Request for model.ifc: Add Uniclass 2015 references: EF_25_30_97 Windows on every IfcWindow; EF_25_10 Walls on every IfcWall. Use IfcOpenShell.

First a look at what the model holds.

```python
import ifcopenshell

model = ifcopenshell.open("model.ifc")
print(model.schema)
print("classifications:", [c.Name for c in model.by_type("IfcClassification")])
for ifc_class in ("IfcDoor", "IfcRoof", "IfcStair", "IfcWall", "IfcWindow"):
    print(ifc_class, len(model.by_type(ifc_class)))
```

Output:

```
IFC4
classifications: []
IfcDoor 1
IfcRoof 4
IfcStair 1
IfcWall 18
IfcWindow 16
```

```python
import ifcopenshell
import ifcopenshell.api.classification

model = ifcopenshell.open("model.ifc")

system = ifcopenshell.api.classification.add_classification(model, classification="Uniclass 2015")

codes = {
    "IfcWindow": ("EF_25_30_97", "Windows"),
    "IfcWall": ("EF_25_10", "Walls"),
}
for ifc_class, (code, name) in codes.items():
    products = model.by_type(ifc_class)
    ifcopenshell.api.classification.add_reference(
        model, products=products, classification=system, identification=code, name=name
    )
    print(code, len(products))

model.write("model_v2.ifc")
```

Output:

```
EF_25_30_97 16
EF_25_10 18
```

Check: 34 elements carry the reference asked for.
